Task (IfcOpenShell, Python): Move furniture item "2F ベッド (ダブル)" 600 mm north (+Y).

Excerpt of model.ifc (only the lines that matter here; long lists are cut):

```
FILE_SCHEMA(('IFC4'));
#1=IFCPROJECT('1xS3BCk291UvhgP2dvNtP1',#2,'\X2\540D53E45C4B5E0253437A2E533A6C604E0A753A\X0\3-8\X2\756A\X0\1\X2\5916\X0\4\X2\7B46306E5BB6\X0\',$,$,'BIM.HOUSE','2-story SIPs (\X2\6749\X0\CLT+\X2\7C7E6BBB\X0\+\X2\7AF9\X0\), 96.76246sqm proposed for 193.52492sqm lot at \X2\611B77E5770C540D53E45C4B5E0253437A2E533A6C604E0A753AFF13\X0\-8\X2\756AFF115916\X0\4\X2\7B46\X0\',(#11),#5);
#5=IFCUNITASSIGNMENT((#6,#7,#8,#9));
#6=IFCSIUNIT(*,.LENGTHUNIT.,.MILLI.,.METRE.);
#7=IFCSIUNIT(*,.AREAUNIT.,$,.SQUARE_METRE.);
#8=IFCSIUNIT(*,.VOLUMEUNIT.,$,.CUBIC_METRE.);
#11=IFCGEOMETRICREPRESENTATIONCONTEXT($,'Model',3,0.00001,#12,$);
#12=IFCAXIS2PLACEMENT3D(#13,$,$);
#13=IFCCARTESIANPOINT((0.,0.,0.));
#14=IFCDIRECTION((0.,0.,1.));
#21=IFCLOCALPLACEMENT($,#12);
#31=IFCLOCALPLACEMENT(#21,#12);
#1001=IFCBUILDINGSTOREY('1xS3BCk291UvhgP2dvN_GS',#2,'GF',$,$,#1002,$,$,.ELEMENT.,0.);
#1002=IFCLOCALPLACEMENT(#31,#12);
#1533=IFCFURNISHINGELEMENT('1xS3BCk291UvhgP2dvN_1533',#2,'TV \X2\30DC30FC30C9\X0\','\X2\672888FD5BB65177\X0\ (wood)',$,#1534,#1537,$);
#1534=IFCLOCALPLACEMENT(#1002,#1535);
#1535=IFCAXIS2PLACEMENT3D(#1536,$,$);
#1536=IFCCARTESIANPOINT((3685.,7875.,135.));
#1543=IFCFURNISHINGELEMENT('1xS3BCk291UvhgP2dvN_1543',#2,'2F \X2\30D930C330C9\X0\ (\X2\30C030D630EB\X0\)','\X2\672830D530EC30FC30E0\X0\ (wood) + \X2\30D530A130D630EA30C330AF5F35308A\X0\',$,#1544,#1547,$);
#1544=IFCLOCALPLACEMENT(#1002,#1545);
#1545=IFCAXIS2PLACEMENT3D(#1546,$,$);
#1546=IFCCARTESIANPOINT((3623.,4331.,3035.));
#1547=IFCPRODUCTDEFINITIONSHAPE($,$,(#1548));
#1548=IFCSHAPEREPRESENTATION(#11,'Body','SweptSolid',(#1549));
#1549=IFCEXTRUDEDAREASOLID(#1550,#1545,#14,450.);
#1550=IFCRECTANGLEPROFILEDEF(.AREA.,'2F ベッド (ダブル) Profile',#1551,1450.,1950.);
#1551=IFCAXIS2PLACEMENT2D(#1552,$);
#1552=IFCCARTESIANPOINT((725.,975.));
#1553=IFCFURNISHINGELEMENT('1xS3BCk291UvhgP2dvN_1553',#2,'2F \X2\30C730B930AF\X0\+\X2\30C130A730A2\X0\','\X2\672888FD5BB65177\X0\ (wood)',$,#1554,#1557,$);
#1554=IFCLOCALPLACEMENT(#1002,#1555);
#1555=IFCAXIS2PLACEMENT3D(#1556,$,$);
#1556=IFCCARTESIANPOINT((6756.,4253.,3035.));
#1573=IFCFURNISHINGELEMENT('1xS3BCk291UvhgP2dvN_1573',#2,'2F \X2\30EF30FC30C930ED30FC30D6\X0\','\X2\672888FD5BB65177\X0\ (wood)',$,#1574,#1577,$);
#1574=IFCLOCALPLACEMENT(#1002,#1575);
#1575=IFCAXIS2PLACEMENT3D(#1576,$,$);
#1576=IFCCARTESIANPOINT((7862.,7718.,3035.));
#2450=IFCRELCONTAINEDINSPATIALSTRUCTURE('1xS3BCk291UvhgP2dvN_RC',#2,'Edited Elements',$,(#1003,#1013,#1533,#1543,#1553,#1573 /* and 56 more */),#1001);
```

```python
import ifcopenshell
import ifcopenshell.api.geometry
import ifcopenshell.util.placement

model = ifcopenshell.open("model.ifc")

item = model.by_id(1543)
matrix = ifcopenshell.util.placement.get_local_placement(item.ObjectPlacement)
matrix[1, 3] += 600.0
ifcopenshell.api.geometry.edit_object_placement(model, product=item, matrix=matrix, is_si=False)

print(ifcopenshell.util.placement.get_local_placement(item.ObjectPlacement).round(3) + 0.0)

model.write("model_edited.ifc")
```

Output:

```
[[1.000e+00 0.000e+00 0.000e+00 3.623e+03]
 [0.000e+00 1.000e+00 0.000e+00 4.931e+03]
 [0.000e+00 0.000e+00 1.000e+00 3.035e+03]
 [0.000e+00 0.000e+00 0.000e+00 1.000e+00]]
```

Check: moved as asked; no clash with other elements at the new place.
